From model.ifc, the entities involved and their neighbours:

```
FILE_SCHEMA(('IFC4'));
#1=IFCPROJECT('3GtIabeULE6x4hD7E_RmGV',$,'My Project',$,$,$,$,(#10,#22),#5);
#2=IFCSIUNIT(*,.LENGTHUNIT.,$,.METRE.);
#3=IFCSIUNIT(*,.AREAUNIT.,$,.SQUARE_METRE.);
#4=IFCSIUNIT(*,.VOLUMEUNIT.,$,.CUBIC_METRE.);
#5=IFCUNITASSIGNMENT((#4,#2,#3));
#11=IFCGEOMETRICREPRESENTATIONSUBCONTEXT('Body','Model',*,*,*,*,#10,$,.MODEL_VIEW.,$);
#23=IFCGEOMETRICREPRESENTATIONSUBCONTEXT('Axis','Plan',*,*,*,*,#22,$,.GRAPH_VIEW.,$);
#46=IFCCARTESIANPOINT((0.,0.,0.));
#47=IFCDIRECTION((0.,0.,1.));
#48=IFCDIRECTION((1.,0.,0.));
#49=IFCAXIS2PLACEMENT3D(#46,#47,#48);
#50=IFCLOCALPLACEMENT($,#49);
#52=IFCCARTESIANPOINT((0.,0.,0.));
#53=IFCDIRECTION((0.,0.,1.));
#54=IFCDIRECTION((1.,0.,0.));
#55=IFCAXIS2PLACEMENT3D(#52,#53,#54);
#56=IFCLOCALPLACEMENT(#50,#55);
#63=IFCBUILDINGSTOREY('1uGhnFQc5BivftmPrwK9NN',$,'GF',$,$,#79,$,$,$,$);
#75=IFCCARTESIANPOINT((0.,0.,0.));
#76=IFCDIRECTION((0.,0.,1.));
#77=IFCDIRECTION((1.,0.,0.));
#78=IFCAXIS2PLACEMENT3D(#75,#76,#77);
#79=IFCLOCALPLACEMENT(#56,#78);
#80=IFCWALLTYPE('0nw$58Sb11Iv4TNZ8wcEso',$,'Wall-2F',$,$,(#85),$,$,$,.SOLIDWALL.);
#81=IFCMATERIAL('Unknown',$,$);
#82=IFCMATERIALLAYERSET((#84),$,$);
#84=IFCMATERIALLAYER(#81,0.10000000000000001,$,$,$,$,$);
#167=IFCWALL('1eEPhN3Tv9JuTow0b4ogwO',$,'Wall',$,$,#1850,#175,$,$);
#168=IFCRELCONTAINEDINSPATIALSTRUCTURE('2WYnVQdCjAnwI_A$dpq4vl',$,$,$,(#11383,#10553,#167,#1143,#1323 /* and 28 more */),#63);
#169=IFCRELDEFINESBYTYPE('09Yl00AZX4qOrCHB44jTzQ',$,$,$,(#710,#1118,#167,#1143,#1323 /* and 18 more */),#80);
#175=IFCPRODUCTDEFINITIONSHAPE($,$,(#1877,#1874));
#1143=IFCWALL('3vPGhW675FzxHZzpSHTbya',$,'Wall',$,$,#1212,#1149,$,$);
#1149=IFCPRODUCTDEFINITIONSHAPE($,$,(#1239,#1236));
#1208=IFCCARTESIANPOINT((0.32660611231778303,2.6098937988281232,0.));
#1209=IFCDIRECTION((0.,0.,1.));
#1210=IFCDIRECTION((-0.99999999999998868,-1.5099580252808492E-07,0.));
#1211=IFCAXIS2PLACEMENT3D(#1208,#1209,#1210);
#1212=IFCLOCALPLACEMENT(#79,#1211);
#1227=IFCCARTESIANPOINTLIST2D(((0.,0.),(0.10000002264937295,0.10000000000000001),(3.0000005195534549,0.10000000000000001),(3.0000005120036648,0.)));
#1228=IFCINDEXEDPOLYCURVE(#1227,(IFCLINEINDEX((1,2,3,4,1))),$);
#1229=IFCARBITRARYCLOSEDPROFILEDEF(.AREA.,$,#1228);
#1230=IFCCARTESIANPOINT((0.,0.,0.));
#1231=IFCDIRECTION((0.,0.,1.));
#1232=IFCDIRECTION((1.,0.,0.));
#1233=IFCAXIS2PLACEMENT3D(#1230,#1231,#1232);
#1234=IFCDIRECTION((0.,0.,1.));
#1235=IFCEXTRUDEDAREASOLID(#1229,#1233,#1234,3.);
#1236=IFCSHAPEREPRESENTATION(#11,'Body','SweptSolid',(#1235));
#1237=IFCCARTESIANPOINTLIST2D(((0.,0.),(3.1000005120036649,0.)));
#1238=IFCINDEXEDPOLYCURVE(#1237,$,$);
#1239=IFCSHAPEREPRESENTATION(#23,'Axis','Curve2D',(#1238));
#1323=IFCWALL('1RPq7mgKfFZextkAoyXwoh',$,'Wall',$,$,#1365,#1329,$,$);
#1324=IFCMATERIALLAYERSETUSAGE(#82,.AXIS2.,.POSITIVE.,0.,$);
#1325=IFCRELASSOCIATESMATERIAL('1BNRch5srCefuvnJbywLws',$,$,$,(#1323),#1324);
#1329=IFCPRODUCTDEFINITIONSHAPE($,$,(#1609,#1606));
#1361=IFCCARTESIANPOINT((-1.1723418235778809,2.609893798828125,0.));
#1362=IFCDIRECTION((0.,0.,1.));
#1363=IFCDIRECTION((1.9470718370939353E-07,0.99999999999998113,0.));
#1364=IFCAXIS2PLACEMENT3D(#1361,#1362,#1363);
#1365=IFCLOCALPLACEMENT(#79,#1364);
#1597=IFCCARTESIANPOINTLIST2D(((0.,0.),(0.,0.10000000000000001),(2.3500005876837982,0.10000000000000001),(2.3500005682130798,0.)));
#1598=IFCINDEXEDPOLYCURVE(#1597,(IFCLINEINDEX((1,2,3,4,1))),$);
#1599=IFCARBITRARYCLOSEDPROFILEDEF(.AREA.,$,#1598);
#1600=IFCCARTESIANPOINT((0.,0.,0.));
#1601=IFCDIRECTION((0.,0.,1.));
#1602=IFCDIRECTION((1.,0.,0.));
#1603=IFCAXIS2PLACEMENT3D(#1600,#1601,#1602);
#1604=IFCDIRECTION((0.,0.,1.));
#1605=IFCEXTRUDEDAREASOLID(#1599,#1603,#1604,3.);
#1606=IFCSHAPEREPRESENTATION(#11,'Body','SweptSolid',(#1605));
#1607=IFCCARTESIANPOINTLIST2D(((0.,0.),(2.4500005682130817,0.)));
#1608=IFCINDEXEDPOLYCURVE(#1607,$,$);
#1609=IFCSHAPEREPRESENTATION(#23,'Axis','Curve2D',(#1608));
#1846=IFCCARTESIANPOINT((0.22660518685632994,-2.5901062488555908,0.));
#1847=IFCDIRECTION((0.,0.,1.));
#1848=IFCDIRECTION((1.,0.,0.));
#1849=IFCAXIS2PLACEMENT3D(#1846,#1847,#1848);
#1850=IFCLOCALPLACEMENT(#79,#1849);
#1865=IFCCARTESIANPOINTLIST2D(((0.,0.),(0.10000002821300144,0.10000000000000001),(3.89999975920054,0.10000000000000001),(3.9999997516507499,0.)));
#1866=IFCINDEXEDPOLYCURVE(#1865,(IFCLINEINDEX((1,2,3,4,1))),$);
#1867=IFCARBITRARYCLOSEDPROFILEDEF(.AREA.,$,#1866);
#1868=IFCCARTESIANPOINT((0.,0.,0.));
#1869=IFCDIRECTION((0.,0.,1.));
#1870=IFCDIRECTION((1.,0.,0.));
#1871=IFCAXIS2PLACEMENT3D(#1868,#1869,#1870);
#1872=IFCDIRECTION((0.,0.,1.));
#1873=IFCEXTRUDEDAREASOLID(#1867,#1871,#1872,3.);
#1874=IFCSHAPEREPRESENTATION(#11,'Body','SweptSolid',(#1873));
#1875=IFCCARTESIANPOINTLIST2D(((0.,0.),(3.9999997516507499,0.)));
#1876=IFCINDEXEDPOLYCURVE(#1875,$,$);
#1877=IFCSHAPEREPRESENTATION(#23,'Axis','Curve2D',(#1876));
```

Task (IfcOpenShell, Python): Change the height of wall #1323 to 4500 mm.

```python
import ifcopenshell
import ifcopenshell.geom
import ifcopenshell.util.representation
import ifcopenshell.util.shape

model = ifcopenshell.open("model.ifc")
settings = ifcopenshell.geom.settings()


def volume(element):
    """Net volume in cubic metres, openings subtracted."""
    shape = ifcopenshell.geom.create_shape(settings, element)
    return ifcopenshell.util.shape.get_volume(shape.geometry)


wall = model.by_guid("1RPq7mgKfFZextkAoyXwoh")
before = volume(wall)

body = ifcopenshell.util.representation.get_representation(wall, "Model", "Body")
solid = body.Items[0]
old_height = solid.Depth
solid.Depth = 4.5
after = volume(wall)

print(f"height {old_height:g} -> {solid.Depth:g}, volume {before:.3f} -> {after:.3f} m3")

model.write("model_edited.ifc")
```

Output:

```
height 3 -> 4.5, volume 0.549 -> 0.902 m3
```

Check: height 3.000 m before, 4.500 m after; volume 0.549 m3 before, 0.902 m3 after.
